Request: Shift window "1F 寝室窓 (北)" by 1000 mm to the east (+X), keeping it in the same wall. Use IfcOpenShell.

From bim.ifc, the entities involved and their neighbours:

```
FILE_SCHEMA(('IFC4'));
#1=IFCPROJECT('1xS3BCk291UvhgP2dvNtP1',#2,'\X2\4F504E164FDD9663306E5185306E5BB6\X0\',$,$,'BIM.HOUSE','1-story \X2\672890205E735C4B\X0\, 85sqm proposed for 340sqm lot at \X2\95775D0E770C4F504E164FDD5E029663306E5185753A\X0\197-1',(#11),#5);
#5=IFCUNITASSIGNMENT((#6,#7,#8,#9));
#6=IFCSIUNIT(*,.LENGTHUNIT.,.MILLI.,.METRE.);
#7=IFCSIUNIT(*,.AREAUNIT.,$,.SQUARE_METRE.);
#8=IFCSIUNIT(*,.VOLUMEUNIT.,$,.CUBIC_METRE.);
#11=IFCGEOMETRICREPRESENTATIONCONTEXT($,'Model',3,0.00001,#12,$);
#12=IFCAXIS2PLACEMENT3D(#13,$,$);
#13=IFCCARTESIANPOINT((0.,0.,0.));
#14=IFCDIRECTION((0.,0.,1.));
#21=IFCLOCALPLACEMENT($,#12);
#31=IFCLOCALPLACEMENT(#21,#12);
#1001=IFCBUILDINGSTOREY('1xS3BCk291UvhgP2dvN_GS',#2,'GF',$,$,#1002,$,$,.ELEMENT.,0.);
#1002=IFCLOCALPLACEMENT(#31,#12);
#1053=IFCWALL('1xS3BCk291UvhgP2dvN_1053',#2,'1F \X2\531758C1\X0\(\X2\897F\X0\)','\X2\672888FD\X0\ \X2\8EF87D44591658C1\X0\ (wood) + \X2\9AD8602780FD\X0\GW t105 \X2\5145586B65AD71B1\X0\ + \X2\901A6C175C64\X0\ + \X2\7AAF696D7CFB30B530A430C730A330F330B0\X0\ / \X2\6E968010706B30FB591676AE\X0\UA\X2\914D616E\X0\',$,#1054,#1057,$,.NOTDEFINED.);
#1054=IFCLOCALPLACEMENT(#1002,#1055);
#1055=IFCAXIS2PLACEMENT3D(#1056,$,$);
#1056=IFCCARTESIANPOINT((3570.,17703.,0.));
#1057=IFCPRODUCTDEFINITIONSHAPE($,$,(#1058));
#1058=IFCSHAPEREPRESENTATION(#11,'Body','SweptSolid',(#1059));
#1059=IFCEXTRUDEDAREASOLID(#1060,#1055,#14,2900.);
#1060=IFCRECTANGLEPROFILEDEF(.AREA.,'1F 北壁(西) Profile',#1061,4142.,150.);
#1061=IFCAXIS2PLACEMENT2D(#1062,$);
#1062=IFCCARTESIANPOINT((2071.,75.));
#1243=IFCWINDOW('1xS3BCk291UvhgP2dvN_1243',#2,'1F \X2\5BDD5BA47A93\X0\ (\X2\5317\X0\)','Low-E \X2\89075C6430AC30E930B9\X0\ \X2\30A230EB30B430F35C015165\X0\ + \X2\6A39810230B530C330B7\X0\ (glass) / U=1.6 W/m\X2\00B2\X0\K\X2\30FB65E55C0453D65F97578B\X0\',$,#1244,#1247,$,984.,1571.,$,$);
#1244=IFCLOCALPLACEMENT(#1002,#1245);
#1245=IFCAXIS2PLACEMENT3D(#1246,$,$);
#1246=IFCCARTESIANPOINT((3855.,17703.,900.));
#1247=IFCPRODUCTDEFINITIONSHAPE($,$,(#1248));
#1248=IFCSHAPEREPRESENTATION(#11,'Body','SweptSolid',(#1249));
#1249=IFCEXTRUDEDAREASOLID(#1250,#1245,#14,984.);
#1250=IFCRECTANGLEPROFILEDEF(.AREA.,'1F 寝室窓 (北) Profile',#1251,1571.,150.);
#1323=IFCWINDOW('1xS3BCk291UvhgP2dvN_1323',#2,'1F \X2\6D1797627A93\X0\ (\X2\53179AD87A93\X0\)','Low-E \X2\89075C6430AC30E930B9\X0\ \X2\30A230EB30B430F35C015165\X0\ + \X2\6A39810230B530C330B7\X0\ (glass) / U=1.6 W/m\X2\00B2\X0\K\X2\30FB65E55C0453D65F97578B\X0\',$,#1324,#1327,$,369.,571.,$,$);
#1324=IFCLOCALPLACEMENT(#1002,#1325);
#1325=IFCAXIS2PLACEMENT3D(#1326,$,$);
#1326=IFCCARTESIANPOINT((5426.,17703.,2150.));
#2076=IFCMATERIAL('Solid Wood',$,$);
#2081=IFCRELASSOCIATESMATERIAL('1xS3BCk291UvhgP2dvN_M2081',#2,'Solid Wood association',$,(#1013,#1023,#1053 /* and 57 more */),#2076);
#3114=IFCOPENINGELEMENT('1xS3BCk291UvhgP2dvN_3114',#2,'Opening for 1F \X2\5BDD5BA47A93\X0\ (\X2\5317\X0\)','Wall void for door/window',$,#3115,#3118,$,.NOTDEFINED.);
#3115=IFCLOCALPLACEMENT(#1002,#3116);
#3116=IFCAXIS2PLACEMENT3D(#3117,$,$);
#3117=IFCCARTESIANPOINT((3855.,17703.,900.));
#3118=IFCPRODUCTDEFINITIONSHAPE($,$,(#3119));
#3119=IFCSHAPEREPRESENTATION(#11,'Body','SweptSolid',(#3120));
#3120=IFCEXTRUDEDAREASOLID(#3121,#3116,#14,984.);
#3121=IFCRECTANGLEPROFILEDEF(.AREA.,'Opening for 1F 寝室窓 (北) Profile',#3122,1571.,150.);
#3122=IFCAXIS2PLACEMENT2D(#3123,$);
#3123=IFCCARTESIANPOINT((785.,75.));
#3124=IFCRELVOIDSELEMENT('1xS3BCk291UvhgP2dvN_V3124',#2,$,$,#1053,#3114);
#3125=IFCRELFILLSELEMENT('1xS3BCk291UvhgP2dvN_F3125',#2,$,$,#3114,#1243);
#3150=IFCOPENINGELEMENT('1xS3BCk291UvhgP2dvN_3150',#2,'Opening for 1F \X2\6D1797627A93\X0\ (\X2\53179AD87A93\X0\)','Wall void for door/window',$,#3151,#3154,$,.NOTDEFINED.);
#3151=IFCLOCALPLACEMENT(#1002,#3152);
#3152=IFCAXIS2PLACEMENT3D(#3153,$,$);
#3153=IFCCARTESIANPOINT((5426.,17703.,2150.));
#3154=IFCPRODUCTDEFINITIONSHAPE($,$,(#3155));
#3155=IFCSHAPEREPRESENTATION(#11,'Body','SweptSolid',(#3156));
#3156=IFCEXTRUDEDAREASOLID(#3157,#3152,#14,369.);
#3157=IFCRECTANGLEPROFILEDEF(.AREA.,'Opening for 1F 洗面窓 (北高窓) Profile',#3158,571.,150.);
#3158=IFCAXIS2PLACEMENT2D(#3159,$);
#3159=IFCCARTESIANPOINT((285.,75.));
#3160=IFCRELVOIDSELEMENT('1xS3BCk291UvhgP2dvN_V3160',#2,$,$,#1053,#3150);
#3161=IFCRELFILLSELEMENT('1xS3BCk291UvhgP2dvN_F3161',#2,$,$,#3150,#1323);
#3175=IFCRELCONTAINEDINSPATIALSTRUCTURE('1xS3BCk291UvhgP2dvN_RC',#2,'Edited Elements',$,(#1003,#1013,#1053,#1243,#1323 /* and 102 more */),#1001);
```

```python
import ifcopenshell
import ifcopenshell.api.geometry
import ifcopenshell.util.placement

model = ifcopenshell.open("bim.ifc")

window = model.by_guid("1xS3BCk291UvhgP2dvN_1243")
opening = window.FillsVoids[0].RelatingOpeningElement
wall = opening.VoidsElements[0].RelatingBuildingElement

wall_matrix = ifcopenshell.util.placement.get_local_placement(wall.ObjectPlacement)
shift = wall_matrix[:3, 0] * 1000.0
before = ifcopenshell.util.placement.get_local_placement(window.ObjectPlacement)[:3, 3].copy()

# The window is not placed relative to its opening, so move both.
for product in (opening, window):
    matrix = ifcopenshell.util.placement.get_local_placement(product.ObjectPlacement)
    matrix[:3, 3] += shift
    ifcopenshell.api.geometry.edit_object_placement(model, product=product, matrix=matrix, is_si=False)

after = ifcopenshell.util.placement.get_local_placement(window.ObjectPlacement)[:3, 3]
print("window moved by", (after - before).round(3) + 0.0)

model.write("bim_v2.ifc")
```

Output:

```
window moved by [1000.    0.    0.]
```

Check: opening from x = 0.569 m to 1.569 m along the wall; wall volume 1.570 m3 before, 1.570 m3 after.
